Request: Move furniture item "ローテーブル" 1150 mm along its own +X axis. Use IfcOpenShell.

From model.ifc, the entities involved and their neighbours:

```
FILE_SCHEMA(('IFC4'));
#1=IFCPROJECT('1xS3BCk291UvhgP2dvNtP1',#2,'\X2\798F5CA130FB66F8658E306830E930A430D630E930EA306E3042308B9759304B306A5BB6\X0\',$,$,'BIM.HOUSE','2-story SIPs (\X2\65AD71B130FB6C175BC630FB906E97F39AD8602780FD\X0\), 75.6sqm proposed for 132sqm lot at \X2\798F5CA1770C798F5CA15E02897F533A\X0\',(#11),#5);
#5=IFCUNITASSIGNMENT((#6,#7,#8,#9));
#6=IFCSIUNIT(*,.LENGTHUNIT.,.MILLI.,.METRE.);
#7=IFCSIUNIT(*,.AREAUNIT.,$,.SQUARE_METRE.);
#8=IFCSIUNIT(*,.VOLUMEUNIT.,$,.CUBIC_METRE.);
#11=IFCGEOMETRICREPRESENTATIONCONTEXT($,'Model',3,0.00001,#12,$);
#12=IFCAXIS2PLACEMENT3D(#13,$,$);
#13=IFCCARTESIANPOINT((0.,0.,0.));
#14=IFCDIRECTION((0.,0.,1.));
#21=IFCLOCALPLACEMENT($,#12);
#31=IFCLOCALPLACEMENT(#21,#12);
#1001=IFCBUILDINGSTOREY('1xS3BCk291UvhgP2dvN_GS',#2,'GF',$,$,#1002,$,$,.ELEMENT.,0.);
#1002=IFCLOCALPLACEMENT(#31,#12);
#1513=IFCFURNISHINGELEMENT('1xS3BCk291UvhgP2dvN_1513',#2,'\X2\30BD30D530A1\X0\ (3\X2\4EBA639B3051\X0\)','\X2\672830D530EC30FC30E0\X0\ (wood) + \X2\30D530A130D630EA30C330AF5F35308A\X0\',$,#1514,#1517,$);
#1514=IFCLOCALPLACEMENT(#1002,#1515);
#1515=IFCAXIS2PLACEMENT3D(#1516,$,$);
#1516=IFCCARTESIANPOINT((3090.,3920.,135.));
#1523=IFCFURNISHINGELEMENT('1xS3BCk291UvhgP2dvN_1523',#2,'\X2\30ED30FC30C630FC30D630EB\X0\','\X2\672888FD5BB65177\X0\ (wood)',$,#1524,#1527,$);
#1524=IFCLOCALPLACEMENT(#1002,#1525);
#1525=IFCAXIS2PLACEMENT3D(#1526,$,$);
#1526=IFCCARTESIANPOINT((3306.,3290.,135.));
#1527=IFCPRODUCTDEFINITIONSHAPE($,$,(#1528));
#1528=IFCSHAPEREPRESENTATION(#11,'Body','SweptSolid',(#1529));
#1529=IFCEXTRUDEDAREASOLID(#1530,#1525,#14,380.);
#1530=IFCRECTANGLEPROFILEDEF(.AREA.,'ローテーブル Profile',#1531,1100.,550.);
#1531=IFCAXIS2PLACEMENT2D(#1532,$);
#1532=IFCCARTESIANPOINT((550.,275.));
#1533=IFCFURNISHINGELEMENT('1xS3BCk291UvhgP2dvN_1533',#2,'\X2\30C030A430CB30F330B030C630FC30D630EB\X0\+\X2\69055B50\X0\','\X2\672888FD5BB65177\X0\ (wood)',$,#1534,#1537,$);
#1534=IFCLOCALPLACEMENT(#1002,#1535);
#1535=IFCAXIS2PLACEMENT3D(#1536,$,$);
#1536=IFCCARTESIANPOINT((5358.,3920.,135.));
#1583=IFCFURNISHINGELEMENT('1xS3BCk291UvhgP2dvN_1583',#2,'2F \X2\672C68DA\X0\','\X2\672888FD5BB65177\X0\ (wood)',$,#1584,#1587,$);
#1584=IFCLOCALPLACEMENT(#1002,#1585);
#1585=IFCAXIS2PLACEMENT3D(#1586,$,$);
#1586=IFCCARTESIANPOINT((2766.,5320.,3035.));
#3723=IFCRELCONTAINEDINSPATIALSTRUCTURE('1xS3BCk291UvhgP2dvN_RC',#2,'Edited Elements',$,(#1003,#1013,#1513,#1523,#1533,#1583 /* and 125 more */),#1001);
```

```python
import ifcopenshell
import ifcopenshell.api.geometry
import ifcopenshell.util.placement
import ifcopenshell.util.unit

model = ifcopenshell.open("model.ifc")
unit_scale = ifcopenshell.util.unit.calculate_unit_scale(model)

item = model.by_guid("1xS3BCk291UvhgP2dvN_1523")
matrix = ifcopenshell.util.placement.get_local_placement(item.ObjectPlacement)
matrix[:3, 3] += matrix[:3, 0] * 1.15 / unit_scale
ifcopenshell.api.geometry.edit_object_placement(model, product=item, matrix=matrix, is_si=False)

print(ifcopenshell.util.placement.get_local_placement(item.ObjectPlacement).round(3) + 0.0)

model.write("model-out.ifc")
```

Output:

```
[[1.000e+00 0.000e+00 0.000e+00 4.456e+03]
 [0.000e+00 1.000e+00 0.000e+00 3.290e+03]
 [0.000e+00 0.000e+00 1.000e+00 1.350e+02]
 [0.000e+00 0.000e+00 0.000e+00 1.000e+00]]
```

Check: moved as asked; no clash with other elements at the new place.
